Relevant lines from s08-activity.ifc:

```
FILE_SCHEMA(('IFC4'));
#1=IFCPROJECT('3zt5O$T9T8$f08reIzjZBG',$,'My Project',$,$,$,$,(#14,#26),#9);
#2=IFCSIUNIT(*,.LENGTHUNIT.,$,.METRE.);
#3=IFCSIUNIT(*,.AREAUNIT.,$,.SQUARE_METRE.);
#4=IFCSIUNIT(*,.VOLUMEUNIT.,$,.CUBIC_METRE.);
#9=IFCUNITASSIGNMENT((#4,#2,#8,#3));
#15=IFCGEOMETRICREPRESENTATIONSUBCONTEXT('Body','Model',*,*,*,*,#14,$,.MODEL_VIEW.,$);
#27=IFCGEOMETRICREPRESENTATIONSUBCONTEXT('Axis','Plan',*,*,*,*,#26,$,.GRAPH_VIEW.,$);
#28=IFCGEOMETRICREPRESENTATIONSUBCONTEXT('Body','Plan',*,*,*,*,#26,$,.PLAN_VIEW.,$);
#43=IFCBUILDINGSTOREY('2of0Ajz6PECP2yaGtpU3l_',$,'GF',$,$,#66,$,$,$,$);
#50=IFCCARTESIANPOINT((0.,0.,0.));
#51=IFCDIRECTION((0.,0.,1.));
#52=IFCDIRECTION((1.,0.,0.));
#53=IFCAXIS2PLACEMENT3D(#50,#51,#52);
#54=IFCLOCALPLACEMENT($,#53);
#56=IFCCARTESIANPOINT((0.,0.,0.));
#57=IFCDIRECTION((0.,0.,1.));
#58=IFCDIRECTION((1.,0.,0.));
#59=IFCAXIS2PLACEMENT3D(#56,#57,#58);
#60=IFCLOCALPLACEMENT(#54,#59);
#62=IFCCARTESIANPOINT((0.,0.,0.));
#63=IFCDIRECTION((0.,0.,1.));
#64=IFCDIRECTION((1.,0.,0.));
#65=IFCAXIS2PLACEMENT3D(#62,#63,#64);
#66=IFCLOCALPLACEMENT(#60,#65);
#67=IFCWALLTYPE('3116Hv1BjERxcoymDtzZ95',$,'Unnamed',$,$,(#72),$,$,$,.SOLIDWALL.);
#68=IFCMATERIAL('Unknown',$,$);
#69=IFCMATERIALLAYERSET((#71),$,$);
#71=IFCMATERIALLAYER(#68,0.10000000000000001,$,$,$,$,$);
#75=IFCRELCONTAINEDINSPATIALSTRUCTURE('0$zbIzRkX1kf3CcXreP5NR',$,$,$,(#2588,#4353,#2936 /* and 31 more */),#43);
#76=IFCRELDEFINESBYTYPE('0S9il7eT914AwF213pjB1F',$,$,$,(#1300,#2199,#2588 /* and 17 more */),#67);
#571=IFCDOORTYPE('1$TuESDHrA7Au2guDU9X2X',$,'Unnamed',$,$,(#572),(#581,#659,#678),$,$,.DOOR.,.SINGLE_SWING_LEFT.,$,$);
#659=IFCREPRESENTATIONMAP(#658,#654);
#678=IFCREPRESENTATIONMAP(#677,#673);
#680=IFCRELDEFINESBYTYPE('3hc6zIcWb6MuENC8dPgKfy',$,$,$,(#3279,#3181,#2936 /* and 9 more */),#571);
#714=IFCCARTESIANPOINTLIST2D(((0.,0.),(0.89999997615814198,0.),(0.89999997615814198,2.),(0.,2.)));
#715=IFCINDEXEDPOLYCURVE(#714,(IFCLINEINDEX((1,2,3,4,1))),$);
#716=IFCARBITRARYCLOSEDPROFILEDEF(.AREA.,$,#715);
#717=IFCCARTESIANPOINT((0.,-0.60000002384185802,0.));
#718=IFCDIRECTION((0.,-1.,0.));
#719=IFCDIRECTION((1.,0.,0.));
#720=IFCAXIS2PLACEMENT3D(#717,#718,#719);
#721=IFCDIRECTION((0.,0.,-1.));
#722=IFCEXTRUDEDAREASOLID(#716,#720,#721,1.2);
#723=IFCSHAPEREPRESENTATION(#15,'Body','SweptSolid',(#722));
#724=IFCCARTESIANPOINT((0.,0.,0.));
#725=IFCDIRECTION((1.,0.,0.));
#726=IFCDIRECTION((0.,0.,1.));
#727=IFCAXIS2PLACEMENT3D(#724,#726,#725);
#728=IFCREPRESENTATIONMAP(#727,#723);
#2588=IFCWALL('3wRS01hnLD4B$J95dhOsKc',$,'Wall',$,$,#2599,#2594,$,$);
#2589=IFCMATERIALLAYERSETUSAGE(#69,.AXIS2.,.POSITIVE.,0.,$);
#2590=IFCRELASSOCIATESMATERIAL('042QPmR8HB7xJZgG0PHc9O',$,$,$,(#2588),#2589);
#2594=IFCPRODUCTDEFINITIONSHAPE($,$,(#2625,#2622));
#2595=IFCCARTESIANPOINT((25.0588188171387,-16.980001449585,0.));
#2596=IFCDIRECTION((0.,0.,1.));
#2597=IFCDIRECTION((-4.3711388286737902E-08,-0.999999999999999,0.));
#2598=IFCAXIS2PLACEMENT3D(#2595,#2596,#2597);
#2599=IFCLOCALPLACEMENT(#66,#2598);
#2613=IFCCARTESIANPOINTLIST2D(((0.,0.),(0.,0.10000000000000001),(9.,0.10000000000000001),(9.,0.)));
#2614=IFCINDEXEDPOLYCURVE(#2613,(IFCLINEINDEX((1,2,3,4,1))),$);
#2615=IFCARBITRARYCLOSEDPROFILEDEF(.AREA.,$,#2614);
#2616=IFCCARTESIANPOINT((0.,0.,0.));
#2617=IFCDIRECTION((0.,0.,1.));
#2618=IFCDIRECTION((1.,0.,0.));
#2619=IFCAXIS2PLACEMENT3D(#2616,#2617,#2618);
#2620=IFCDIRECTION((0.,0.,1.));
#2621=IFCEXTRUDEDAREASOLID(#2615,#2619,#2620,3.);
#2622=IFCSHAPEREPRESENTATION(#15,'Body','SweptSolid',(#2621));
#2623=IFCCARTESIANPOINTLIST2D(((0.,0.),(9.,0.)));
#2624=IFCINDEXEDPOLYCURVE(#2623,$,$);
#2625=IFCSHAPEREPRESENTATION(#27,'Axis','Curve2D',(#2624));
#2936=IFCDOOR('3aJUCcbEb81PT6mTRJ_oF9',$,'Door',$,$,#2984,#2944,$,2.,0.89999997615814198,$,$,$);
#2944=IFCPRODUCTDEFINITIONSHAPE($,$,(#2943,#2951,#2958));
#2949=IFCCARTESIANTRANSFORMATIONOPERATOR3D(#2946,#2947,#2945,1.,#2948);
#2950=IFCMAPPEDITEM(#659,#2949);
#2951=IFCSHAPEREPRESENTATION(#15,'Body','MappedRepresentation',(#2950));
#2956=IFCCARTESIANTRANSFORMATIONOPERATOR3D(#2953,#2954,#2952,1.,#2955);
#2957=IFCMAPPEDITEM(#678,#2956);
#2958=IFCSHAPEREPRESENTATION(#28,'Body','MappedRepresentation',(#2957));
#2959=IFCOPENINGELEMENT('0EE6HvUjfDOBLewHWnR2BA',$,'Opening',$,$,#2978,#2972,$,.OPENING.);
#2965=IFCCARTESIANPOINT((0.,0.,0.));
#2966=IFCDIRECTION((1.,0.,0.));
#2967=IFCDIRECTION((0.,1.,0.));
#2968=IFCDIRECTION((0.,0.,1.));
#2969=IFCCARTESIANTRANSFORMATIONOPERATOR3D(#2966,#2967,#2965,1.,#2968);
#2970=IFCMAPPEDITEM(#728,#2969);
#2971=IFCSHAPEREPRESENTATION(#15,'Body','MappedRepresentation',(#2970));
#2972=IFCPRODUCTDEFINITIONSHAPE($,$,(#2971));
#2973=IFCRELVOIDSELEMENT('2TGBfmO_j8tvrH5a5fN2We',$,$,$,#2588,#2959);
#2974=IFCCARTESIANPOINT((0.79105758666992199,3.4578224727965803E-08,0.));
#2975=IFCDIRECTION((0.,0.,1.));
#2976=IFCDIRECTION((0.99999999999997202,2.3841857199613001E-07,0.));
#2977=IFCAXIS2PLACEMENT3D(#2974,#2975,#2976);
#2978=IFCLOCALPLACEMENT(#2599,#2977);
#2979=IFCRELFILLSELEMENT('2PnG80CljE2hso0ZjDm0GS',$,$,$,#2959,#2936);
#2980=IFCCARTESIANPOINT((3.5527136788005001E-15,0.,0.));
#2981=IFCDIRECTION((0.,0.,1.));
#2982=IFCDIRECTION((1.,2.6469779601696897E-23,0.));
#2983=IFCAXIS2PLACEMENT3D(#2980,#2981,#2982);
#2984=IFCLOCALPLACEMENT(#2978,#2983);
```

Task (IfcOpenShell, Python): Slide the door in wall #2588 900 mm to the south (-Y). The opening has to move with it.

```python
import ifcopenshell
import ifcopenshell.api.geometry
import ifcopenshell.util.placement

model = ifcopenshell.open("s08-activity.ifc")

door = model.by_guid("3aJUCcbEb81PT6mTRJ_oF9")
opening = door.FillsVoids[0].RelatingOpeningElement
wall = opening.VoidsElements[0].RelatingBuildingElement

wall_matrix = ifcopenshell.util.placement.get_local_placement(wall.ObjectPlacement)
shift = wall_matrix[:3, 0] * 0.9
before = ifcopenshell.util.placement.get_local_placement(door.ObjectPlacement)[:3, 3].copy()

# The door is placed relative to its opening, so it follows when the opening moves.
matrix = ifcopenshell.util.placement.get_local_placement(opening.ObjectPlacement)
matrix[:3, 3] += shift
ifcopenshell.api.geometry.edit_object_placement(
    model, product=opening, matrix=matrix, is_si=False, should_transform_children=True
)

after = ifcopenshell.util.placement.get_local_placement(door.ObjectPlacement)[:3, 3]
print("door moved by", (after - before).round(3) + 0.0)

model.write("s08-activity_updated.ifc")
```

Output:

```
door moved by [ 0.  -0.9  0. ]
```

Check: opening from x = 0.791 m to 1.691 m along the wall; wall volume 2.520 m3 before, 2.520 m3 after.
